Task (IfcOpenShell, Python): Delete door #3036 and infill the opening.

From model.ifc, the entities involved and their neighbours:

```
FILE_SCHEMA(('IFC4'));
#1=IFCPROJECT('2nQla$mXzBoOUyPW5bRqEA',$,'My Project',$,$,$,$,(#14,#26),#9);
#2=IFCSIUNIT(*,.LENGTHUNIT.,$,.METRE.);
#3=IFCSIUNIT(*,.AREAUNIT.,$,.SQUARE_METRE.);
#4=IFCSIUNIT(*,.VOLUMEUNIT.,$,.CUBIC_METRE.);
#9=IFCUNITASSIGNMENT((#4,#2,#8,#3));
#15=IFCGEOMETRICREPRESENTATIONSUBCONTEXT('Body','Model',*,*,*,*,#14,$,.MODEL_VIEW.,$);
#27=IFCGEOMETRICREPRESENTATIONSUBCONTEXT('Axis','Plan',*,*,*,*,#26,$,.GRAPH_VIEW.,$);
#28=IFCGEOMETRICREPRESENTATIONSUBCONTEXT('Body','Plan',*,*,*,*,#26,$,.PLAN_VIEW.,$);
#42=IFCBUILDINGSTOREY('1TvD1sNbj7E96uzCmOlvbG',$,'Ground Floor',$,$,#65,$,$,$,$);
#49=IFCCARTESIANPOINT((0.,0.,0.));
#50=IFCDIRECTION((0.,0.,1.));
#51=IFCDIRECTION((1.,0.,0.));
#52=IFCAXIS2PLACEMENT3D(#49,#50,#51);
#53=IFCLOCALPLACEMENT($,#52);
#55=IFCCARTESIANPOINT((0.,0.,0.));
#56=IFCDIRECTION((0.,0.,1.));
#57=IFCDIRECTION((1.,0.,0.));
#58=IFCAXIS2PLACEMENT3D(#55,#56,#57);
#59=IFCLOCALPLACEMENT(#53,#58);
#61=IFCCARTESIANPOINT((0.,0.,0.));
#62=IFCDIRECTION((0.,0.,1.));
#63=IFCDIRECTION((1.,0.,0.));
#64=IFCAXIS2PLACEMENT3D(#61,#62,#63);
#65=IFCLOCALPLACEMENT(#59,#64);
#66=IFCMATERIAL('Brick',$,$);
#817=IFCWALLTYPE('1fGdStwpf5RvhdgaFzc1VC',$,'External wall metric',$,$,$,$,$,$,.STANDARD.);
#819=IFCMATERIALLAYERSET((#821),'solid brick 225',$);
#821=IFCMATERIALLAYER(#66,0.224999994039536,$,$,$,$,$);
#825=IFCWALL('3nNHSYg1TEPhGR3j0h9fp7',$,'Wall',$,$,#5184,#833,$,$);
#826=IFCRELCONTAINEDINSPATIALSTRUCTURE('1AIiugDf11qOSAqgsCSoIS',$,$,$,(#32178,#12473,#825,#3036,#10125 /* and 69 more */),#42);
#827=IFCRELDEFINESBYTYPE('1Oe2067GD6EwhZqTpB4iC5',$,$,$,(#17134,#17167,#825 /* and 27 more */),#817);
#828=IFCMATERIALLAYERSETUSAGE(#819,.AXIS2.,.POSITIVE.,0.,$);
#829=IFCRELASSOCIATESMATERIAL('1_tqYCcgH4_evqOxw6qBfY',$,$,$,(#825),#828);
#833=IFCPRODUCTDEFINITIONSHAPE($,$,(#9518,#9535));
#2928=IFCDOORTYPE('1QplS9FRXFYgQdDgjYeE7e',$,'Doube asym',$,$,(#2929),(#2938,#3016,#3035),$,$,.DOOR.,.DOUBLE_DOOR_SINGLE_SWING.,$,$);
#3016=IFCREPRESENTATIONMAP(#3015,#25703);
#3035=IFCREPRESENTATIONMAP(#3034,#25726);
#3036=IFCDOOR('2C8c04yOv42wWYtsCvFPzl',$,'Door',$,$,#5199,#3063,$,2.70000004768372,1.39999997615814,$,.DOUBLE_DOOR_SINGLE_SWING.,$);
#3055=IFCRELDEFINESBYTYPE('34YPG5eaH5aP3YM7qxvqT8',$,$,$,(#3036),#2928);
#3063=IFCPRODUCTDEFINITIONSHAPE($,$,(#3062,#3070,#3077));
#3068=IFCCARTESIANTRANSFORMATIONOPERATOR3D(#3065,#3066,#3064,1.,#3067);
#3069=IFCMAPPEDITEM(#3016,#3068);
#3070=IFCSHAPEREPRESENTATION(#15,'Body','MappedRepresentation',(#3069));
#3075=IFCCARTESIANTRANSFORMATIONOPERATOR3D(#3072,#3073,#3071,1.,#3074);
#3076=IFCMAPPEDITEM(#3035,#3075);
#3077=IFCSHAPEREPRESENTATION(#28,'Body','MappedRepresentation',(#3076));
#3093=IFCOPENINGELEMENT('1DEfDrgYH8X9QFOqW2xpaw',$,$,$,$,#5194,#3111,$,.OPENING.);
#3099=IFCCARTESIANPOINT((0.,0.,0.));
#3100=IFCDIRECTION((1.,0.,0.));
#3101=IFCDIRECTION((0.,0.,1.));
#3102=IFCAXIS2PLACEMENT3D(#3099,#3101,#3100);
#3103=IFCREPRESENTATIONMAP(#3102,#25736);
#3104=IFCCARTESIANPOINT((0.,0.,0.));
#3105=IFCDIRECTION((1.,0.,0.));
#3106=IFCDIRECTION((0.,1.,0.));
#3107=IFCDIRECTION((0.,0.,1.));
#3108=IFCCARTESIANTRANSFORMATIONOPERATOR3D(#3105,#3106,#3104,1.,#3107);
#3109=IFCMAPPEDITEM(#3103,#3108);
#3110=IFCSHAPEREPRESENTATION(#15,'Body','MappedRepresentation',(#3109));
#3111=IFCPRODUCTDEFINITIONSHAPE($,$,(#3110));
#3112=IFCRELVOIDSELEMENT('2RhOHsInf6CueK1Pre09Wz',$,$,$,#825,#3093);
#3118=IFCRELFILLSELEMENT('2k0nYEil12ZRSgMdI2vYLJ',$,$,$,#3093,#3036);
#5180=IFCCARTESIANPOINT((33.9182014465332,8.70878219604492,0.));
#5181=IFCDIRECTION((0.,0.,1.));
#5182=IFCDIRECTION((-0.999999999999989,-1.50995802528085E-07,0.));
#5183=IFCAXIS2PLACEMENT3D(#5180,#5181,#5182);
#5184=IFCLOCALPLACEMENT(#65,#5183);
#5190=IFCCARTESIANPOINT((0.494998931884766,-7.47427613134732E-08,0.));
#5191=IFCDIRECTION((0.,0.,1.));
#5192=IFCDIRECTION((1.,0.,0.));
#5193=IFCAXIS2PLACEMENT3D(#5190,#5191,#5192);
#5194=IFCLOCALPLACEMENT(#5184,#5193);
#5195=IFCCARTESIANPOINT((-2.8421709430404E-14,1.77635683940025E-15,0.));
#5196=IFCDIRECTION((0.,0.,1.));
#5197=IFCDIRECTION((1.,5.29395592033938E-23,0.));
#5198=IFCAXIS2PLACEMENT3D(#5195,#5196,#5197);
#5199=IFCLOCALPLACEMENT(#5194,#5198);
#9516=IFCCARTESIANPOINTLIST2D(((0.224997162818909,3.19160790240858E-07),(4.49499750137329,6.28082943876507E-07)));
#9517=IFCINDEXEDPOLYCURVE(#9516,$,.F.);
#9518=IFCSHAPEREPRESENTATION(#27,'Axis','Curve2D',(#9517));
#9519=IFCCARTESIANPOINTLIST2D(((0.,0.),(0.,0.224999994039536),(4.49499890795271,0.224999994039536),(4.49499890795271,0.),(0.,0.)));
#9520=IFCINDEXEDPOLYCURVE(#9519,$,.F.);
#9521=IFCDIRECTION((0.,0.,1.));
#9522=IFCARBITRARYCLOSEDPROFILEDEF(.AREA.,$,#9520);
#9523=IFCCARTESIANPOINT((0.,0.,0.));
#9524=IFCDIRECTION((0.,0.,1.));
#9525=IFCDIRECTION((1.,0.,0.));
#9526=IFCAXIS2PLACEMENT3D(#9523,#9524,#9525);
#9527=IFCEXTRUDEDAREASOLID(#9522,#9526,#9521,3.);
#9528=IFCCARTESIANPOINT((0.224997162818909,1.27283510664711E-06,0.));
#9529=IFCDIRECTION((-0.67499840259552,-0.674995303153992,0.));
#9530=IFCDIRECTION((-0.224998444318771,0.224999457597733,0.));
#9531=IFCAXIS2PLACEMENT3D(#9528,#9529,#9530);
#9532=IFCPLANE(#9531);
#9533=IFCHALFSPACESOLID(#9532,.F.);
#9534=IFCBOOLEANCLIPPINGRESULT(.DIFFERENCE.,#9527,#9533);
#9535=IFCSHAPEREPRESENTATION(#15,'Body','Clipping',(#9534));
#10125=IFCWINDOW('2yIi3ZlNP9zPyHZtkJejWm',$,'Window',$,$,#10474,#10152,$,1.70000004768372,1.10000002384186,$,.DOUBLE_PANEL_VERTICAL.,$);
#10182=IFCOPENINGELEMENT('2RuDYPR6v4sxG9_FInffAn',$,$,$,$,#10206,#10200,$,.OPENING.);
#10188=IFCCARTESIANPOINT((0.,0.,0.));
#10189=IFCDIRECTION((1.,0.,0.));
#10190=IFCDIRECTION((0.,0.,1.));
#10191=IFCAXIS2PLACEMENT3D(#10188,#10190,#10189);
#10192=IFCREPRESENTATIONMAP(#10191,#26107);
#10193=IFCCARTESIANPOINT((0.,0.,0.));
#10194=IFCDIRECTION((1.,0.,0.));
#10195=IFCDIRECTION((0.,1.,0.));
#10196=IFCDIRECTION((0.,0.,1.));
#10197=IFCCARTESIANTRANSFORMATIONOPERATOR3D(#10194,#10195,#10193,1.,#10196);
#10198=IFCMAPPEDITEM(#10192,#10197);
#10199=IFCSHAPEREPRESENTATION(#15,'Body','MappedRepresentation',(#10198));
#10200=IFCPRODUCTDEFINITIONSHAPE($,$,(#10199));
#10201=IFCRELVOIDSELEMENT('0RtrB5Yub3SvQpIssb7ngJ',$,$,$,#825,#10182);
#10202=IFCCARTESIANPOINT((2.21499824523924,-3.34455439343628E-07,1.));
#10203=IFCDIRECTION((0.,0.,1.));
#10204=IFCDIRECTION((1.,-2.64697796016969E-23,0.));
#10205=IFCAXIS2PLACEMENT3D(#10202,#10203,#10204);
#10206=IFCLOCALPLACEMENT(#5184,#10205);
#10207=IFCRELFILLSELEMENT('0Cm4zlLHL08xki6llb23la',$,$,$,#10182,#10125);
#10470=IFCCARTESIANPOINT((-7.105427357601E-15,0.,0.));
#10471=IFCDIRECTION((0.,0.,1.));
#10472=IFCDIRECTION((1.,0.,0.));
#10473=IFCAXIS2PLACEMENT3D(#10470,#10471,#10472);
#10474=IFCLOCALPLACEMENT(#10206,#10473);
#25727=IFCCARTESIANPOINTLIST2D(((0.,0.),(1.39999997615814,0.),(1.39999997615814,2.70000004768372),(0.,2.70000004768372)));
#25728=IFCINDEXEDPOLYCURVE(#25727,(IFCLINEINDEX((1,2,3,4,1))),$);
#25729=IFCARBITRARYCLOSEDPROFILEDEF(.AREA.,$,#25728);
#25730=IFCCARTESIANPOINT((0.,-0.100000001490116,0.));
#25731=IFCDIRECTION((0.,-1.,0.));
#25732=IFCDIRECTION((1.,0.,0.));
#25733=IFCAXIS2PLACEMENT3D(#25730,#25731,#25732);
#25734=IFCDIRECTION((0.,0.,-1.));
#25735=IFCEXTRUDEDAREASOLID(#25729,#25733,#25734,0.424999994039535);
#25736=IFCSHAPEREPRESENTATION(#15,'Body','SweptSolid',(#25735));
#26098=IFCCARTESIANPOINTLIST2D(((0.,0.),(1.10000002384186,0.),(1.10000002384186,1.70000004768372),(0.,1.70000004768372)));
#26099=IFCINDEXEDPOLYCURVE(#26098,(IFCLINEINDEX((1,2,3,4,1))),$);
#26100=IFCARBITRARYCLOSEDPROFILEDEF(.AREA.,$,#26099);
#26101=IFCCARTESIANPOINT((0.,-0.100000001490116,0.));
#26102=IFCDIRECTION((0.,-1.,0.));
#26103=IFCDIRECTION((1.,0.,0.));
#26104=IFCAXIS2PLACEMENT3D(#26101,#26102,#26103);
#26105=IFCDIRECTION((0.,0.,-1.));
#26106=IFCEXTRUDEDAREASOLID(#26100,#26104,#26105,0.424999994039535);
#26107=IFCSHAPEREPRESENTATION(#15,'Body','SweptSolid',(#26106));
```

```python
import ifcopenshell
import ifcopenshell.api.feature
import ifcopenshell.api.root
import ifcopenshell.geom
import ifcopenshell.util.shape

model = ifcopenshell.open("model.ifc")
settings = ifcopenshell.geom.settings()


def volume(element):
    """Net volume in cubic metres, openings subtracted."""
    shape = ifcopenshell.geom.create_shape(settings, element)
    return ifcopenshell.util.shape.get_volume(shape.geometry)


door = model.by_id(3036)
opening = door.FillsVoids[0].RelatingOpeningElement
wall = opening.VoidsElements[0].RelatingBuildingElement
before = volume(wall)

ifcopenshell.api.root.remove_product(model, product=door)
ifcopenshell.api.feature.remove_feature(model, feature=opening)

after = volume(wall)

print(f"wall volume {before:.3f} -> {after:.3f} m3")

model.write("model_rev.ifc")
```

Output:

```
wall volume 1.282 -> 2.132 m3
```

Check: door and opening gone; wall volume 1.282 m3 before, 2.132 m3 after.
